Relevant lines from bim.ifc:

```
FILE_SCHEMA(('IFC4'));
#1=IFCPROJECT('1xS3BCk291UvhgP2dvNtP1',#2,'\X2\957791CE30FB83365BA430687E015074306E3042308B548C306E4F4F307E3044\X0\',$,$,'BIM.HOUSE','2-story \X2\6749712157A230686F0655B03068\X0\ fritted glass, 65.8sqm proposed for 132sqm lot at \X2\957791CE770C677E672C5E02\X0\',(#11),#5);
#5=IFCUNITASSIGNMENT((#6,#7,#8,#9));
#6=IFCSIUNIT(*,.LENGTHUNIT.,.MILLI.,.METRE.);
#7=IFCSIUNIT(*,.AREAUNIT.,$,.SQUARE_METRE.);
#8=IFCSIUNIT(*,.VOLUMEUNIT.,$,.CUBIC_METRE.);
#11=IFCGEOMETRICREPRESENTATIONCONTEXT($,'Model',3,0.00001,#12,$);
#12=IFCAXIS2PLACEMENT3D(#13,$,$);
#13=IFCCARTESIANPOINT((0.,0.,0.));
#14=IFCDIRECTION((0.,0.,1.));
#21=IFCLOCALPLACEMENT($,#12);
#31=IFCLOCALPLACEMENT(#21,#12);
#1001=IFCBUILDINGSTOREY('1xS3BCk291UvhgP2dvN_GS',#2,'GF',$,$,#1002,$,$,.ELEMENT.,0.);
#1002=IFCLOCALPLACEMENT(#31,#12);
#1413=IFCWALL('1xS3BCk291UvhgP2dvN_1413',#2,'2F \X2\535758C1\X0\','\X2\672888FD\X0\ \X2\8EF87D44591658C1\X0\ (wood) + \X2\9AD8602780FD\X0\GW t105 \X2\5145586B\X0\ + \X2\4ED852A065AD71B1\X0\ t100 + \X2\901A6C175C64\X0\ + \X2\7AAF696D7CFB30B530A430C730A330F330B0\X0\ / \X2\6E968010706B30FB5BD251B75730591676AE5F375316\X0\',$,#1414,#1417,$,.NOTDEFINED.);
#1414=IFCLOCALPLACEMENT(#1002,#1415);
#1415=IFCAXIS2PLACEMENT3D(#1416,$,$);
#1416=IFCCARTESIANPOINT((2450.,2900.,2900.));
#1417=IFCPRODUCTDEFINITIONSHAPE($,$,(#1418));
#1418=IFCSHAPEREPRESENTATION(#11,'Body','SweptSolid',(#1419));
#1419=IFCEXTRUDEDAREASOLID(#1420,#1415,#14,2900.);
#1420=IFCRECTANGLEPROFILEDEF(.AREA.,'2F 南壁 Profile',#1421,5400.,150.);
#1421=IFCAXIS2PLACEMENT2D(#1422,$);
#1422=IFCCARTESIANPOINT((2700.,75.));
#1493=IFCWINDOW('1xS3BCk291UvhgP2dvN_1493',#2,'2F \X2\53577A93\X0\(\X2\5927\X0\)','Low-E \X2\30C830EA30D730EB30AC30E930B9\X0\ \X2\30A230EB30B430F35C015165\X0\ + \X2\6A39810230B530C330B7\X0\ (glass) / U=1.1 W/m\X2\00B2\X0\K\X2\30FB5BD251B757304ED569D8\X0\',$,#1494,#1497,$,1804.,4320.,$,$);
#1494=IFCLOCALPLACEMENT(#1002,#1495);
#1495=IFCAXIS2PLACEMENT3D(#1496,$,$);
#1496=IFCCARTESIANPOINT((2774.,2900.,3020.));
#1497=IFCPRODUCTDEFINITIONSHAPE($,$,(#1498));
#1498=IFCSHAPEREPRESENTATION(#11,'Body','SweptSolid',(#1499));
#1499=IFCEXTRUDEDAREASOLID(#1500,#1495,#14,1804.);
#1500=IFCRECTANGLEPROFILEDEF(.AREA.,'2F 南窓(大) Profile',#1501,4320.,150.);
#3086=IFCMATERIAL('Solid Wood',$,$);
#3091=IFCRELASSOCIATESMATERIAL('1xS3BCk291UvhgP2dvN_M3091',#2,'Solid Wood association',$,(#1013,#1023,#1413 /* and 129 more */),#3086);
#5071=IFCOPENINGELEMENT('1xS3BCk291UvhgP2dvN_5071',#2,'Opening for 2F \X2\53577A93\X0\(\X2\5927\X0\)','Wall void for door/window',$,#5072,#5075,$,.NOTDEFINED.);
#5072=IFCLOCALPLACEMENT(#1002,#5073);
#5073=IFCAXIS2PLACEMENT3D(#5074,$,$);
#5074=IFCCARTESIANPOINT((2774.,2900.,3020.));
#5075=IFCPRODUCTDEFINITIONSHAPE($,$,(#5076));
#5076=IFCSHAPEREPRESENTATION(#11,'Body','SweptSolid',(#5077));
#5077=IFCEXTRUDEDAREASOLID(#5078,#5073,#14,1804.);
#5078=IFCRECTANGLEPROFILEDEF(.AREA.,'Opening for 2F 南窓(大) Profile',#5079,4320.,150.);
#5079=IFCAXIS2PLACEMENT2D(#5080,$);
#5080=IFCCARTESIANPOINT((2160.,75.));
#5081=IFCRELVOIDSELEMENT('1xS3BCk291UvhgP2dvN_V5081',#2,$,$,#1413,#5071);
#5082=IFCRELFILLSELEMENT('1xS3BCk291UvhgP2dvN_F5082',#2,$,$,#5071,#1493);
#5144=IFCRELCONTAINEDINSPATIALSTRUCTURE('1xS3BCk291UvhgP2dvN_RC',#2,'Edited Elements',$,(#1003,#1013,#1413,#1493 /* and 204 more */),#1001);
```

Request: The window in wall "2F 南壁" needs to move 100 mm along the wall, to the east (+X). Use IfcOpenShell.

```python
import ifcopenshell
import ifcopenshell.api.geometry
import ifcopenshell.util.placement
import ifcopenshell.util.unit

model = ifcopenshell.open("bim.ifc")
unit_scale = ifcopenshell.util.unit.calculate_unit_scale(model)

window = model.by_guid("1xS3BCk291UvhgP2dvN_1493")
opening = window.FillsVoids[0].RelatingOpeningElement
wall = opening.VoidsElements[0].RelatingBuildingElement

wall_matrix = ifcopenshell.util.placement.get_local_placement(wall.ObjectPlacement)
shift = wall_matrix[:3, 0] * 0.1 / unit_scale
before = ifcopenshell.util.placement.get_local_placement(window.ObjectPlacement)[:3, 3].copy()

# The window is not placed relative to its opening, so move both.
for product in (opening, window):
    matrix = ifcopenshell.util.placement.get_local_placement(product.ObjectPlacement)
    matrix[:3, 3] += shift
    ifcopenshell.api.geometry.edit_object_placement(model, product=product, matrix=matrix, is_si=False)

after = ifcopenshell.util.placement.get_local_placement(window.ObjectPlacement)[:3, 3]
print("window moved by", (after - before).round(3) + 0.0)

model.write("bim-out.ifc")
```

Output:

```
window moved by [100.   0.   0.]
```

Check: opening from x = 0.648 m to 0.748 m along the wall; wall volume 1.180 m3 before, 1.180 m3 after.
